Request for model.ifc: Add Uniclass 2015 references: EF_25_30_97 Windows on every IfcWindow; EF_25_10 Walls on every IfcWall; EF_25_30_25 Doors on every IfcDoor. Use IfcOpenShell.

First a look at what the model holds.

```python
import ifcopenshell

model = ifcopenshell.open("model.ifc")
print(model.schema)
print("classifications:", [c.Name for c in model.by_type("IfcClassification")])
for ifc_class in ("IfcDoor", "IfcRoof", "IfcStair", "IfcWall", "IfcWindow"):
    print(ifc_class, len(model.by_type(ifc_class)))
```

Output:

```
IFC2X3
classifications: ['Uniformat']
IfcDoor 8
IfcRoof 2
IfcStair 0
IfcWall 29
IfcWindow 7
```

```python
import ifcopenshell
import ifcopenshell.api.classification

model = ifcopenshell.open("model.ifc")

# IFC2X3 requires Source and Edition and has no link from the project to the system.
system = model.create_entity("IfcClassification", Source="NBS", Edition="2015", Name="Uniclass 2015")

codes = {
    "IfcWindow": ("EF_25_30_97", "Windows"),
    "IfcWall": ("EF_25_10", "Walls"),
    "IfcDoor": ("EF_25_30_25", "Doors"),
}
for ifc_class, (code, name) in codes.items():
    products = model.by_type(ifc_class)
    ifcopenshell.api.classification.add_reference(
        model, products=products, classification=system, identification=code, name=name
    )
    print(code, len(products))

model.write("model_updated.ifc")
```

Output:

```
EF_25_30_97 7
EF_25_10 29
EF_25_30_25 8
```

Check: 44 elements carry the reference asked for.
